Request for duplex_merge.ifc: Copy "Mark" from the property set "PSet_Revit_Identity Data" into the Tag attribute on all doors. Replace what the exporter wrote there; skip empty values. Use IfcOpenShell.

First a look at what the model holds.

```python
import ifcopenshell
import ifcopenshell.util.element

model = ifcopenshell.open("duplex_merge.ifc")
print(model.schema)
doors = model.by_type("IfcDoor")
print(len(doors), "doors")
for e in doors[:8]:
    source = ifcopenshell.util.element.get_pset(e, "PSet_Revit_Identity Data", "Mark")
    target = e.Tag
    print(e.id(), repr(source), repr(target), sep=" | ")
```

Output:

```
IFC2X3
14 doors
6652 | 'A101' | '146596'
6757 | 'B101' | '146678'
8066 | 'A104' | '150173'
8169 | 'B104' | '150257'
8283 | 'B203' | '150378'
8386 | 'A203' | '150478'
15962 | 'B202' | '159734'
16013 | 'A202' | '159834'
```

```python
import ifcopenshell
import ifcopenshell.util.element

model = ifcopenshell.open("duplex_merge.ifc")

count = 0
for e in model.by_type("IfcDoor"):
    value = ifcopenshell.util.element.get_pset(e, "PSet_Revit_Identity Data", "Mark")
    current = e.Tag
    if not value or not value.strip() or current == value:
        continue
    e.Tag = value
    count += 1

print(count, "doors updated")

model.write("duplex_merge_edited.ifc")
```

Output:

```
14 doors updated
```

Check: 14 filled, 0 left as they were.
